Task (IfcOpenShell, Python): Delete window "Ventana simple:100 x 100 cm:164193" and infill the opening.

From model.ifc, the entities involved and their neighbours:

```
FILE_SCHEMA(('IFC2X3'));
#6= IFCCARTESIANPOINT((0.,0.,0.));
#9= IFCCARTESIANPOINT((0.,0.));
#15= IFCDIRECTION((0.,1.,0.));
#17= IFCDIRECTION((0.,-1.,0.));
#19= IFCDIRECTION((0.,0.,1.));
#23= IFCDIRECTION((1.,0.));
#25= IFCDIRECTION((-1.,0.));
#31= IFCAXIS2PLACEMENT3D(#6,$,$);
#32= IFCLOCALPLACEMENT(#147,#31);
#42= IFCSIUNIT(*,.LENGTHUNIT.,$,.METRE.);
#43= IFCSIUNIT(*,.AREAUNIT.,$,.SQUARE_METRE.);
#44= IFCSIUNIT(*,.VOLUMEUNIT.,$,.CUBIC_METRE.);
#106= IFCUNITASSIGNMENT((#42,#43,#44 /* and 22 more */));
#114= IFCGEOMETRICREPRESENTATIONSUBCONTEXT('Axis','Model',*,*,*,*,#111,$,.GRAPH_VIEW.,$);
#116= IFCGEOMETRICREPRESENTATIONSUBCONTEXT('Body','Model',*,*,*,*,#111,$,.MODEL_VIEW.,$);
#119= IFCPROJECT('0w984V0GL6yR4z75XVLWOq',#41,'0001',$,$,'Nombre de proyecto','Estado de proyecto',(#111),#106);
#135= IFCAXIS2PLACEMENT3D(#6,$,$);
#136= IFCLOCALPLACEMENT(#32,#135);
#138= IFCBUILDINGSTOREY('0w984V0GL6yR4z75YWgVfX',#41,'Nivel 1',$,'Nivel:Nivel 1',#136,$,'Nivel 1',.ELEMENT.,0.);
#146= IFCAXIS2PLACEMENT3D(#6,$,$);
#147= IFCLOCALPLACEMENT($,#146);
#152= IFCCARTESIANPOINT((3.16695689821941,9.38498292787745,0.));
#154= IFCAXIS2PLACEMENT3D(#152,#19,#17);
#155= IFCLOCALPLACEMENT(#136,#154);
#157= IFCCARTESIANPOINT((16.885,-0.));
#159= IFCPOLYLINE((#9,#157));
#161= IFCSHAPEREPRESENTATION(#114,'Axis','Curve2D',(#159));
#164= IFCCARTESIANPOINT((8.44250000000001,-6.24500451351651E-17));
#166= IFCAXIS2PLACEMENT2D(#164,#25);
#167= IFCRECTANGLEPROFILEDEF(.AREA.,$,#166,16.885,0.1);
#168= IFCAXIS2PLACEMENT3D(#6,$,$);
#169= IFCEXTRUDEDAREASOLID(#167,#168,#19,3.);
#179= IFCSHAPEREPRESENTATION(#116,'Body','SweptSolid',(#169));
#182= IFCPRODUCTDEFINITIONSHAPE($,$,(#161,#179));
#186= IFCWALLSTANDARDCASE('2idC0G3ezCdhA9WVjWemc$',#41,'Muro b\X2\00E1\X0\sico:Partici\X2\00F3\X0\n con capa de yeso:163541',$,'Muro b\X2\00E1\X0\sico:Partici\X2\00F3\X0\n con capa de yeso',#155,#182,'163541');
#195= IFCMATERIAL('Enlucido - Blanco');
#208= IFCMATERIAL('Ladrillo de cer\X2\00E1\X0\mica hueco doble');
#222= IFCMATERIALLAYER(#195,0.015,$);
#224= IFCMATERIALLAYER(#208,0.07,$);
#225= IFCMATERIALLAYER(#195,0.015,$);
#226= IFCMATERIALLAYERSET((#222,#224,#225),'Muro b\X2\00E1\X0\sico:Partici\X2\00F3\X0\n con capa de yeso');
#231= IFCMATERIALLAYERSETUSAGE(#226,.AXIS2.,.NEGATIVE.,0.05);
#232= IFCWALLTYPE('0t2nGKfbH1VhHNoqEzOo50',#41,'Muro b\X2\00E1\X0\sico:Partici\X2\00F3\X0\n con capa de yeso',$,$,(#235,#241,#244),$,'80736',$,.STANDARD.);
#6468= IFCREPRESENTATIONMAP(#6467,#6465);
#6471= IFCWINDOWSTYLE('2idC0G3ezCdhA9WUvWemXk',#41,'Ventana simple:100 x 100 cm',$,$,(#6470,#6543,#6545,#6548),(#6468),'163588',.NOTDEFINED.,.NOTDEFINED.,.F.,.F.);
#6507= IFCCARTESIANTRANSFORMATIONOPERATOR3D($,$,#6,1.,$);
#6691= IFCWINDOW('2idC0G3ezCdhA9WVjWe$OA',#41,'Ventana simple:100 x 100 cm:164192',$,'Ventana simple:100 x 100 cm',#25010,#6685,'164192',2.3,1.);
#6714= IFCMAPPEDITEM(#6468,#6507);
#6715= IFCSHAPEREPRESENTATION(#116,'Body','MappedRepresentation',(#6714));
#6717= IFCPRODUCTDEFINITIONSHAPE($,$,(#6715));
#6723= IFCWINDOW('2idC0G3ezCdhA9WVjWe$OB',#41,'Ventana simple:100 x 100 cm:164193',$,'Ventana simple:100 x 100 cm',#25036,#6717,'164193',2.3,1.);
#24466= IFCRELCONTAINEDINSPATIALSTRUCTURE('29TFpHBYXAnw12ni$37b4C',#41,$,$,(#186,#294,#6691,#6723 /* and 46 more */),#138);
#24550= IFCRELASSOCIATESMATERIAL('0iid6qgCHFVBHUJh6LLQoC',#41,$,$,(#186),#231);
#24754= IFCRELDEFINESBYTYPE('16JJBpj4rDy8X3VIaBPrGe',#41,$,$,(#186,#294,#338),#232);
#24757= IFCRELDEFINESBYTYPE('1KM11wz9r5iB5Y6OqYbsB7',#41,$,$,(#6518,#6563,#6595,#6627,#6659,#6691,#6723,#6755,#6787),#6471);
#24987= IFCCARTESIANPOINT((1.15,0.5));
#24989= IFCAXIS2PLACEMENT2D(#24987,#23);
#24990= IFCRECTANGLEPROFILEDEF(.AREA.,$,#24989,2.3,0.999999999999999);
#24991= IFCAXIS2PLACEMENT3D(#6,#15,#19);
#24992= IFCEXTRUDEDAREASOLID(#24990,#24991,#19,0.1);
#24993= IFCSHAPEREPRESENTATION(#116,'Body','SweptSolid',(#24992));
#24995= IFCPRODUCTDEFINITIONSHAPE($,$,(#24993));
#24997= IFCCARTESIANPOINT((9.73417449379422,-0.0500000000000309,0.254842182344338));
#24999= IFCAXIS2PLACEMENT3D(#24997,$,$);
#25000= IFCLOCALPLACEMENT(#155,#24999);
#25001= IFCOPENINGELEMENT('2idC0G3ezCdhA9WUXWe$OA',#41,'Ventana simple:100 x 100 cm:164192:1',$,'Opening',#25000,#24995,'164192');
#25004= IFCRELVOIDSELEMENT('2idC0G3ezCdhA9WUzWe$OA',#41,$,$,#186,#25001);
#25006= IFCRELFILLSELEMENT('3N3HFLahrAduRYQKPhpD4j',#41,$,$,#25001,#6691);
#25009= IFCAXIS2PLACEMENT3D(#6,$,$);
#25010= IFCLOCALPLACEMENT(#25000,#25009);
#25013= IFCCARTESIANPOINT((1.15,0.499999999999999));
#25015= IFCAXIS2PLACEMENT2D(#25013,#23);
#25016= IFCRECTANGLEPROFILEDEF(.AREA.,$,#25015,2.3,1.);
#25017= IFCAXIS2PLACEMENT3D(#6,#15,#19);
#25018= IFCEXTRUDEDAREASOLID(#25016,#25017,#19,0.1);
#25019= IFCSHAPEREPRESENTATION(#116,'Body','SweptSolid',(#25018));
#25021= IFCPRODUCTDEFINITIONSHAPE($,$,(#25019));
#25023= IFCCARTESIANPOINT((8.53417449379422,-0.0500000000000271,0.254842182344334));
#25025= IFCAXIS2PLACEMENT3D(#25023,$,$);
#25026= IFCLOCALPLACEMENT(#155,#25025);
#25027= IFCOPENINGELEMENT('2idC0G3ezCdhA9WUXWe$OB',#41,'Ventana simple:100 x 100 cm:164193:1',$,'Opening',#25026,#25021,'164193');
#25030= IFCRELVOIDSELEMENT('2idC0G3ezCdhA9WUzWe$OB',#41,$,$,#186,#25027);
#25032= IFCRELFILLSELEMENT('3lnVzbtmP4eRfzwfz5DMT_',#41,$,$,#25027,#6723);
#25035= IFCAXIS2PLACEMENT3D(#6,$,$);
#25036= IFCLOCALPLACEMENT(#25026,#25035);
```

```python
import ifcopenshell
import ifcopenshell.api.feature
import ifcopenshell.api.root
import ifcopenshell.geom
import ifcopenshell.util.shape

model = ifcopenshell.open("model.ifc")
settings = ifcopenshell.geom.settings()


def volume(element):
    """Net volume in cubic metres, openings subtracted."""
    shape = ifcopenshell.geom.create_shape(settings, element)
    return ifcopenshell.util.shape.get_volume(shape.geometry)


window = model.by_guid("2idC0G3ezCdhA9WVjWe$OB")
opening = window.FillsVoids[0].RelatingOpeningElement
wall = opening.VoidsElements[0].RelatingBuildingElement
before = volume(wall)

ifcopenshell.api.root.remove_product(model, product=window)
ifcopenshell.api.feature.remove_feature(model, feature=opening)

after = volume(wall)

print(f"wall volume {before:.3f} -> {after:.3f} m3")

model.write("model_edited.ifc")
```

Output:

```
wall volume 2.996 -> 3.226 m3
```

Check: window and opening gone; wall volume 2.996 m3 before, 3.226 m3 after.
